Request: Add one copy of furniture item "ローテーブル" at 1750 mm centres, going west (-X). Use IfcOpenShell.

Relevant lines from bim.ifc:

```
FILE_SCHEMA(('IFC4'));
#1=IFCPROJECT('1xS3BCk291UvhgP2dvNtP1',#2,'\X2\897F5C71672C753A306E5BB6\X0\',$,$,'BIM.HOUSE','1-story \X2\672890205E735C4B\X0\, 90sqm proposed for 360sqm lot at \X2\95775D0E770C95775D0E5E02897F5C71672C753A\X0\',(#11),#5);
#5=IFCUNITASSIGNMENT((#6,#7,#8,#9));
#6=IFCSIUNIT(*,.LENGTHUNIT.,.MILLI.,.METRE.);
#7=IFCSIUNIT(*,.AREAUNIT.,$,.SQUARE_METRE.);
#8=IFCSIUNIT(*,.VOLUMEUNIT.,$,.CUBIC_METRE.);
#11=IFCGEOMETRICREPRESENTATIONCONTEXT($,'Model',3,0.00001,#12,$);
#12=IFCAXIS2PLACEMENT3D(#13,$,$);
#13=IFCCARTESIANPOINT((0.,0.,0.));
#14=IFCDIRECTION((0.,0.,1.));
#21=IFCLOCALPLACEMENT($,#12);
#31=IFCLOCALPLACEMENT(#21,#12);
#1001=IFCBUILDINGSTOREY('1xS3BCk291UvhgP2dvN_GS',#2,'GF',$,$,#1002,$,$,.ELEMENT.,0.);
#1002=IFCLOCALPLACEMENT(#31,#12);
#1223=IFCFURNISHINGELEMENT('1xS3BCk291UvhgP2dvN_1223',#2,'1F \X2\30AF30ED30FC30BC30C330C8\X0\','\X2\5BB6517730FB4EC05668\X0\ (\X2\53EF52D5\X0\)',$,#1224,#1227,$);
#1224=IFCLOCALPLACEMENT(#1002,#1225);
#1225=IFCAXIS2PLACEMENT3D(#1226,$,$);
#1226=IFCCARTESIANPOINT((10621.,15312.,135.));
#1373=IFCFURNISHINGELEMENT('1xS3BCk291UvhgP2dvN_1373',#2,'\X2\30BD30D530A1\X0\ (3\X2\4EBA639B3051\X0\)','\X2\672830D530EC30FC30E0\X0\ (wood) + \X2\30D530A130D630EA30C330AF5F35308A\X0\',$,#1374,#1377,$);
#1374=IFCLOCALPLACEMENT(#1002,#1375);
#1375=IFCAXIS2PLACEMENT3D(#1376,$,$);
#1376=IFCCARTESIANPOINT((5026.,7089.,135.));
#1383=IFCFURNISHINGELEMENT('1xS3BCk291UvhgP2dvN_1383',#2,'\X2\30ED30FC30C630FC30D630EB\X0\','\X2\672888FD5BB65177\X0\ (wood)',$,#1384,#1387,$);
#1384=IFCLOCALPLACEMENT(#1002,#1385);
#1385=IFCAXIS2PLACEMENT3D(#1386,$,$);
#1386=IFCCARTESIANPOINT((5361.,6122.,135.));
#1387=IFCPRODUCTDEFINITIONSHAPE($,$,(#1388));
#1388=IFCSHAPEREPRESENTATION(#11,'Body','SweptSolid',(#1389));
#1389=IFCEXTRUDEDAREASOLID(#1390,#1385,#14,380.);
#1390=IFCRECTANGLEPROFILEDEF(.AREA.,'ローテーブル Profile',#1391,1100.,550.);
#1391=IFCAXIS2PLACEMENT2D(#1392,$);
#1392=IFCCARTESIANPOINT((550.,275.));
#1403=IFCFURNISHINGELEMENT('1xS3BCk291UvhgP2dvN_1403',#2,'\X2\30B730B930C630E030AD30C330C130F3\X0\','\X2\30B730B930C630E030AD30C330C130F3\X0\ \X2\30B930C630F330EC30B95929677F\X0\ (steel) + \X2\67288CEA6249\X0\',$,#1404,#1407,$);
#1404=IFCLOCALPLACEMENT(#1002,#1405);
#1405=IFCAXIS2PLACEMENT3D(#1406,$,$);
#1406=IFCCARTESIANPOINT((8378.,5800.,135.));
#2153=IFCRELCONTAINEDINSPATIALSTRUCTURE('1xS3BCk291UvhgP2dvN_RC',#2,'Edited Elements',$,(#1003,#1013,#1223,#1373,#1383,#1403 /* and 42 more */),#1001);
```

```python
import numpy as np
import ifcopenshell
import ifcopenshell.api.geometry
import ifcopenshell.api.root
import ifcopenshell.util.element
import ifcopenshell.util.placement
import ifcopenshell.util.unit

model = ifcopenshell.open("bim.ifc")
unit_scale = ifcopenshell.util.unit.calculate_unit_scale(model)


def reuse_history(source, copy):
    """copy_class also copies each property set's owner history, people and application; keep the originals."""
    for rel in copy.IsDefinedBy:
        if rel.is_a("IfcRelDefinesByProperties") and (history := rel.RelatingPropertyDefinition.OwnerHistory):
            rel.RelatingPropertyDefinition.OwnerHistory = source.OwnerHistory
            ifcopenshell.util.element.remove_deep2(model, history)


source = model.by_guid("1xS3BCk291UvhgP2dvN_1383")
base = ifcopenshell.util.placement.get_local_placement(source.ObjectPlacement)
step = np.array([-1.0, 0.0, 0.0]) * 1.75 / unit_scale

for i in range(1, 2):
    copy = ifcopenshell.api.root.copy_class(model, product=source)
    copy.Representation = ifcopenshell.util.element.copy_deep(
        model, source.Representation, exclude=["IfcGeometricRepresentationContext", "IfcRepresentationMap"]
    )
    reuse_history(source, copy)
    matrix = base.copy()
    matrix[:3, 3] += i * step
    print("added at", matrix[:3, 3].round(3) + 0.0)
    ifcopenshell.api.geometry.edit_object_placement(model, product=copy, matrix=matrix, is_si=False)

model.write("bim_edited.ifc")
```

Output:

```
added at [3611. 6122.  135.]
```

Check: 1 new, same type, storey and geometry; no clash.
